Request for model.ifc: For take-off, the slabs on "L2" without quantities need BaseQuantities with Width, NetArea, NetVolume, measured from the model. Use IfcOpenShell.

First a look at what the model holds.

```python
import ifcopenshell
import ifcopenshell.util.element
import ifcopenshell.util.unit

model = ifcopenshell.open("model.ifc")
print(model.schema)
for unit_type in ("LENGTHUNIT", "AREAUNIT", "VOLUMEUNIT"):
    print(unit_type, ifcopenshell.util.unit.calculate_unit_scale(model, unit_type))
storey = next(s for s in model.by_type("IfcBuildingStorey") if s.Name == "L2")
slabs = [e for e in ifcopenshell.util.element.get_decomposition(storey) if e.is_a("IfcSlab")]
for e in sorted(slabs, key=lambda e: e.id()):
    print(e.id(), e.is_a(), e.Name, list(ifcopenshell.util.element.get_psets(e, qtos_only=True)), sep=" | ")
```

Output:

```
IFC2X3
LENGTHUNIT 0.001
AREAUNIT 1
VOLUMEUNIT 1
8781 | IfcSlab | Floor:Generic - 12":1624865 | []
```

```python
import ifcopenshell
import ifcopenshell.api.pset
import ifcopenshell.geom
import ifcopenshell.util.element
import ifcopenshell.util.shape
import ifcopenshell.util.unit

model = ifcopenshell.open("model.ifc")
unit_scale = ifcopenshell.util.unit.calculate_unit_scale(model)
area_scale = ifcopenshell.util.unit.calculate_unit_scale(model, "AREAUNIT")
volume_scale = ifcopenshell.util.unit.calculate_unit_scale(model, "VOLUMEUNIT")
settings = ifcopenshell.geom.settings()

storey = next(s for s in model.by_type("IfcBuildingStorey") if s.Name == "L2")
slabs = [e for e in ifcopenshell.util.element.get_decomposition(storey) if e.is_a("IfcSlab")]

for e in sorted(slabs, key=lambda e: e.id()):
    if ifcopenshell.util.element.get_psets(e, qtos_only=True, should_inherit=False):
        continue
    # Geometry comes back in metres, in the element's own axes.
    shape = ifcopenshell.geom.create_shape(settings, e)
    values = {
        "Width": ifcopenshell.util.shape.get_z(shape.geometry) / unit_scale,
        "NetArea": ifcopenshell.util.shape.get_footprint_area(shape.geometry) / area_scale,
        "NetVolume": ifcopenshell.util.shape.get_volume(shape.geometry) / volume_scale,
    }
    qto = ifcopenshell.api.pset.add_qto(model, product=e, name="BaseQuantities")
    ifcopenshell.api.pset.edit_qto(model, qto=qto, properties=values)
    print(e.id(), {k: round(v, 3) for k, v in values.items()})

model.write("model_v2.ifc")
```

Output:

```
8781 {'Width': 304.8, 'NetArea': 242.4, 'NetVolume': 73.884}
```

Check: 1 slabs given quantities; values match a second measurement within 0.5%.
